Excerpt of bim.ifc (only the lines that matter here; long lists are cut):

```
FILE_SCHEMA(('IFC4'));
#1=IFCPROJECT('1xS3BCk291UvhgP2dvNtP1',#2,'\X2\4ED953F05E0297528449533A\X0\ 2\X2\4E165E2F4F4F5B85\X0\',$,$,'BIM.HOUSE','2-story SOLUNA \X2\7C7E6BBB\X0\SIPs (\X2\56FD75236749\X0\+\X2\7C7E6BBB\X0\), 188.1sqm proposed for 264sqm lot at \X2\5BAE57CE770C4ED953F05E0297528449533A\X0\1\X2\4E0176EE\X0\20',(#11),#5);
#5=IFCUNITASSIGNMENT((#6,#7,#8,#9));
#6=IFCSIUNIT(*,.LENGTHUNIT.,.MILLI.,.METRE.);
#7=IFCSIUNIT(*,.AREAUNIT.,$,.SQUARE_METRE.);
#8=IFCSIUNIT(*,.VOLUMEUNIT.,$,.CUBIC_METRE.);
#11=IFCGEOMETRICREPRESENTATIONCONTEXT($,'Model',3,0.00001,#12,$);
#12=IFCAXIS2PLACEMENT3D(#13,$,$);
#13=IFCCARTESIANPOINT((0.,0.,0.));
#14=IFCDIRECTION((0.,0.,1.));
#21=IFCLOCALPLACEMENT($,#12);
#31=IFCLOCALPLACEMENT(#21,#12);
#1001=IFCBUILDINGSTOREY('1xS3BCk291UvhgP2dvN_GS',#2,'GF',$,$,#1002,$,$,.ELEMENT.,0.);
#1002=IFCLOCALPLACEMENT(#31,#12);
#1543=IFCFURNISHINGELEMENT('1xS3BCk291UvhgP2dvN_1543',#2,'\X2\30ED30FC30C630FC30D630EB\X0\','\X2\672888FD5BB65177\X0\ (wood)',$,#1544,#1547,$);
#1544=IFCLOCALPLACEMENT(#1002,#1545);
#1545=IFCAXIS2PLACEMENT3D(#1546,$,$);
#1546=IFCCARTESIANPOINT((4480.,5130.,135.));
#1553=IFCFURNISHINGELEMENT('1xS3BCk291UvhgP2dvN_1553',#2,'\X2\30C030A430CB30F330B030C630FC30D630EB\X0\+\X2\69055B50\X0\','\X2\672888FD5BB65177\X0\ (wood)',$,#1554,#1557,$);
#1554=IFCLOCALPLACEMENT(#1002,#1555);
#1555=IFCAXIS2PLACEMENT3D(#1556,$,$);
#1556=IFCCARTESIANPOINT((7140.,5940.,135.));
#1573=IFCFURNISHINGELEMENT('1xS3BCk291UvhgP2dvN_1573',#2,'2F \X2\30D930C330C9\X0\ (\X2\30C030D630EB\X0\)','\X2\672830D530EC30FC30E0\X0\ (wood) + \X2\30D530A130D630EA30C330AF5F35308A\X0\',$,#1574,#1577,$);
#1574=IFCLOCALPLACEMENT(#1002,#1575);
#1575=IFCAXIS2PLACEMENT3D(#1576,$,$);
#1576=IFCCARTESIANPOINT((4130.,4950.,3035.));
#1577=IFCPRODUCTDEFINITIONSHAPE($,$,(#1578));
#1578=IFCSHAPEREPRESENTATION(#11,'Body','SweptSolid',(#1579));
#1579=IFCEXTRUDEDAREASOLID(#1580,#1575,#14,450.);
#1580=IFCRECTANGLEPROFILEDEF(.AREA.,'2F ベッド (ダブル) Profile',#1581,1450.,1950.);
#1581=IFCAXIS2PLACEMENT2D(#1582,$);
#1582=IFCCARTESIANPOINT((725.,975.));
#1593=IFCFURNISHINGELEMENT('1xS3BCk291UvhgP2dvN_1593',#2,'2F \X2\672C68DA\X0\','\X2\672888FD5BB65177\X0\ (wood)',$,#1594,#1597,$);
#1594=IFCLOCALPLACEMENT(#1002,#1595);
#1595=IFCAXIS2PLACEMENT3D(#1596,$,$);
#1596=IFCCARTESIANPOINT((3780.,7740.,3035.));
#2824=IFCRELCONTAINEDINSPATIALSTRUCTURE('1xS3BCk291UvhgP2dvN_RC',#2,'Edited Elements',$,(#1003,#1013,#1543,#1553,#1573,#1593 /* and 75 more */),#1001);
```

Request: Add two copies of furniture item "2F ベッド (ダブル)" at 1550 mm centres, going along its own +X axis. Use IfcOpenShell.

```python
import ifcopenshell
import ifcopenshell.api.geometry
import ifcopenshell.api.root
import ifcopenshell.util.element
import ifcopenshell.util.placement
import ifcopenshell.util.unit

model = ifcopenshell.open("bim.ifc")
unit_scale = ifcopenshell.util.unit.calculate_unit_scale(model)


def reuse_history(source, copy):
    """copy_class also copies each property set's owner history, people and application; keep the originals."""
    for rel in copy.IsDefinedBy:
        if rel.is_a("IfcRelDefinesByProperties") and (history := rel.RelatingPropertyDefinition.OwnerHistory):
            rel.RelatingPropertyDefinition.OwnerHistory = source.OwnerHistory
            ifcopenshell.util.element.remove_deep2(model, history)


source = model.by_guid("1xS3BCk291UvhgP2dvN_1573")
base = ifcopenshell.util.placement.get_local_placement(source.ObjectPlacement)
step = base[:3, 0] * 1.55 / unit_scale

for i in range(1, 3):
    copy = ifcopenshell.api.root.copy_class(model, product=source)
    copy.Representation = ifcopenshell.util.element.copy_deep(
        model, source.Representation, exclude=["IfcGeometricRepresentationContext", "IfcRepresentationMap"]
    )
    reuse_history(source, copy)
    matrix = base.copy()
    matrix[:3, 3] += i * step
    print("added at", matrix[:3, 3].round(3) + 0.0)
    ifcopenshell.api.geometry.edit_object_placement(model, product=copy, matrix=matrix, is_si=False)

model.write("bim_rev.ifc")
```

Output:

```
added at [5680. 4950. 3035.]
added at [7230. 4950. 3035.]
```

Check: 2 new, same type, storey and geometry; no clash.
